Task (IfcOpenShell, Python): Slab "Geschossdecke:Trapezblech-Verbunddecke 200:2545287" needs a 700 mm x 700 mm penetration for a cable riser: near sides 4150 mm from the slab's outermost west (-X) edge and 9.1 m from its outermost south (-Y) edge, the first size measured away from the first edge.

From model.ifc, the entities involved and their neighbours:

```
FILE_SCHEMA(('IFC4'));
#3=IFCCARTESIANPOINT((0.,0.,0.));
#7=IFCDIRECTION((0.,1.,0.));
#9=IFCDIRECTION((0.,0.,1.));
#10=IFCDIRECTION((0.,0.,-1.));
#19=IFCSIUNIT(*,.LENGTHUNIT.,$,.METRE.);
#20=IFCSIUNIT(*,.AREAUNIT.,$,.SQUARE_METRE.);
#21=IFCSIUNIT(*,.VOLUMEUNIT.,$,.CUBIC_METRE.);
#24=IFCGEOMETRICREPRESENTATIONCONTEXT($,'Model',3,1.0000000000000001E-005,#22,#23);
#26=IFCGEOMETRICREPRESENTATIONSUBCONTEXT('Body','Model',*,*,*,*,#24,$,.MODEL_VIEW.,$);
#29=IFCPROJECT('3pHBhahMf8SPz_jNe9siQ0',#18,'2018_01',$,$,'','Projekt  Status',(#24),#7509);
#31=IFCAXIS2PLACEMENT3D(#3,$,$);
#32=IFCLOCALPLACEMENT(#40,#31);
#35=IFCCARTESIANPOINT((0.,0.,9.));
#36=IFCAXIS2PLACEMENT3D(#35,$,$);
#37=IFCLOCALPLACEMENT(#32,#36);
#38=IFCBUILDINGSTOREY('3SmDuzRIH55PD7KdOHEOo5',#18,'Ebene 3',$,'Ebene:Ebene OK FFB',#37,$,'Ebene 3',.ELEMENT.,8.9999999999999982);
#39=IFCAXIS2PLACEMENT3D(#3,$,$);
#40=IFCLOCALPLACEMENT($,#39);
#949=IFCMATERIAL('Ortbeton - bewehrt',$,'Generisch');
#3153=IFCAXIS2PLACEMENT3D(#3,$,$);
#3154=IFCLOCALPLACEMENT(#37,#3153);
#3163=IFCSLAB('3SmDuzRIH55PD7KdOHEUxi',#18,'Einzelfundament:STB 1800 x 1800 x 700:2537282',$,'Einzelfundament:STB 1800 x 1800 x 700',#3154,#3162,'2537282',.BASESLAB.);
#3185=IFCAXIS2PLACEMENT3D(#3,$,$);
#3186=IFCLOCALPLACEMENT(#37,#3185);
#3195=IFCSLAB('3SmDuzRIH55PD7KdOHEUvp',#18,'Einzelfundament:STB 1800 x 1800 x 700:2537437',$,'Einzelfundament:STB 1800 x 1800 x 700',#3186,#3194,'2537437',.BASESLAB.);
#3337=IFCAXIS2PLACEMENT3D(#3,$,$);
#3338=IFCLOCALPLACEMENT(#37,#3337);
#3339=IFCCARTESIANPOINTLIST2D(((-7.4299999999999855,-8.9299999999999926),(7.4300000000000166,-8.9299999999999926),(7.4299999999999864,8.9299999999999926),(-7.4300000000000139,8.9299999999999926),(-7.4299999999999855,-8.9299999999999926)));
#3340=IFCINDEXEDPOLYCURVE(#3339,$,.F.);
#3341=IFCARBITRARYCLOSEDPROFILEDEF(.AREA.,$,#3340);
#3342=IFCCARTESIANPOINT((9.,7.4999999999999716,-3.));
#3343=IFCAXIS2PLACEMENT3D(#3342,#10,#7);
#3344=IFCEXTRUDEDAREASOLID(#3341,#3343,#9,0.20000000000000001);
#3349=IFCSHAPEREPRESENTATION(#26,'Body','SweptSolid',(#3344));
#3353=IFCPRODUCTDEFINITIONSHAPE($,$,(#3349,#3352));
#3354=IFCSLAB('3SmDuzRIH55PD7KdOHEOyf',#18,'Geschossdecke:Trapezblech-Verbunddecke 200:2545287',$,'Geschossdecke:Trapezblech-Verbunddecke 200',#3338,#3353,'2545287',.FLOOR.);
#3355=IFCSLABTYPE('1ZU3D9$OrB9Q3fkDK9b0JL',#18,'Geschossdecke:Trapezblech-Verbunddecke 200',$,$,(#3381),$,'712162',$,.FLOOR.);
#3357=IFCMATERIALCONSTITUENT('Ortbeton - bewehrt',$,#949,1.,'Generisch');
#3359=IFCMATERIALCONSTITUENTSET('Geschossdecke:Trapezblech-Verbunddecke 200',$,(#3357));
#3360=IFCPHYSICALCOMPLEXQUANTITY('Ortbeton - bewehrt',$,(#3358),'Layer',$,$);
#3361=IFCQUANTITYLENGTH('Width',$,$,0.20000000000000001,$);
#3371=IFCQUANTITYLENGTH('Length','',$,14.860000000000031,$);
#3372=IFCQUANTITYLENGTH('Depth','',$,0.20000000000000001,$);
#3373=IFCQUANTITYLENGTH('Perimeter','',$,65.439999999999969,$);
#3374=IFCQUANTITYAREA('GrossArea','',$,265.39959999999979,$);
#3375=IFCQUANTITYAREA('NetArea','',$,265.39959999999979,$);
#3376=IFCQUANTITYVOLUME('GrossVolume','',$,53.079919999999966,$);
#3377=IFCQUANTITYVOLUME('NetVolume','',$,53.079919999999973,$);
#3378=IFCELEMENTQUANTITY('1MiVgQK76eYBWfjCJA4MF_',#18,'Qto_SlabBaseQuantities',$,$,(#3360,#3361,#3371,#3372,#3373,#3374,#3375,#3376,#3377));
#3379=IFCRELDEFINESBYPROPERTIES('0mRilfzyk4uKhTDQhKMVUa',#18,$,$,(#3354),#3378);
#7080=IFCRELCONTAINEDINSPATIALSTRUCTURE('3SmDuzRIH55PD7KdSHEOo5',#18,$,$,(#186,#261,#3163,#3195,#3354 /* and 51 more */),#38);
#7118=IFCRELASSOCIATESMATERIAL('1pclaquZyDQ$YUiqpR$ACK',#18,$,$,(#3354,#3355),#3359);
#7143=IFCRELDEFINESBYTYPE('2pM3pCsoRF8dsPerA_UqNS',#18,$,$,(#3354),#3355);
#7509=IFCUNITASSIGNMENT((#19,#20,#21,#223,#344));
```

```python
import numpy as np
import ifcopenshell
import ifcopenshell.api.feature
import ifcopenshell.api.geometry
import ifcopenshell.api.pset
import ifcopenshell.api.root
import ifcopenshell.geom
import ifcopenshell.util.element
import ifcopenshell.util.placement
import ifcopenshell.util.representation
import ifcopenshell.util.shape
import ifcopenshell.util.unit

model = ifcopenshell.open("model.ifc")
unit_scale = ifcopenshell.util.unit.calculate_unit_scale(model)
area_scale = ifcopenshell.util.unit.calculate_unit_scale(model, "AREAUNIT")
volume_scale = ifcopenshell.util.unit.calculate_unit_scale(model, "VOLUMEUNIT")
settings = ifcopenshell.geom.settings()


def volume(element):
    """Net volume in cubic metres, openings subtracted."""
    shape = ifcopenshell.geom.create_shape(settings, element)
    return ifcopenshell.util.shape.get_volume(shape.geometry)


slab = model.by_guid("3SmDuzRIH55PD7KdOHEOyf")
before = volume(slab)

# Extent in the slab's own axes, in metres. The edges named are its -X and -Y sides.
slab_shape = ifcopenshell.geom.create_shape(settings, slab)
vertices = ifcopenshell.util.shape.get_vertices(slab_shape.geometry)
x_min, y_min, bottom = vertices.min(axis=0)
top = vertices[:, 2].max()

opening = ifcopenshell.api.root.create_entity(model, ifc_class="IfcOpeningElement", name="Cable riser opening", predefined_type="OPENING")
context = ifcopenshell.util.representation.get_context(model, "Model", "Body", "MODEL_VIEW")
width, depth = 0.7, 0.7
outline = [(0.0, 0.0), (width, 0.0), (width, depth), (0.0, depth), (0.0, 0.0)]
# Overshoot both faces by 50 mm so the cut is clean.
shape = ifcopenshell.api.geometry.add_slab_representation(
    model, context=context, depth=top - bottom + 0.1, polyline=outline
)
ifcopenshell.api.geometry.assign_representation(model, product=opening, representation=shape)

matrix = ifcopenshell.util.placement.get_local_placement(slab.ObjectPlacement)
matrix[:, 3] = matrix @ np.append(np.array([x_min + 4.15, y_min + 9.1, bottom - 0.05]) / unit_scale, 1.0)
ifcopenshell.api.geometry.edit_object_placement(model, product=opening, matrix=matrix, is_si=False)
ifcopenshell.api.feature.add_feature(model, feature=opening, element=slab)

after = volume(slab)

# Update the slab's stored quantities.
qto = model.by_id(ifcopenshell.util.element.get_pset(slab, "Qto_SlabBaseQuantities", should_inherit=False)["id"])
ifcopenshell.api.pset.edit_qto(model, qto=qto, properties={
    "NetArea": after / (top - bottom) / area_scale,
    "NetVolume": after / volume_scale,
})

print(f"slab volume {before:.3f} -> {after:.3f} m3")

model.write("model_rev.ifc")
```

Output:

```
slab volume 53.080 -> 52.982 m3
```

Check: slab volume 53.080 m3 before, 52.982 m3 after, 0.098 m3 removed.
